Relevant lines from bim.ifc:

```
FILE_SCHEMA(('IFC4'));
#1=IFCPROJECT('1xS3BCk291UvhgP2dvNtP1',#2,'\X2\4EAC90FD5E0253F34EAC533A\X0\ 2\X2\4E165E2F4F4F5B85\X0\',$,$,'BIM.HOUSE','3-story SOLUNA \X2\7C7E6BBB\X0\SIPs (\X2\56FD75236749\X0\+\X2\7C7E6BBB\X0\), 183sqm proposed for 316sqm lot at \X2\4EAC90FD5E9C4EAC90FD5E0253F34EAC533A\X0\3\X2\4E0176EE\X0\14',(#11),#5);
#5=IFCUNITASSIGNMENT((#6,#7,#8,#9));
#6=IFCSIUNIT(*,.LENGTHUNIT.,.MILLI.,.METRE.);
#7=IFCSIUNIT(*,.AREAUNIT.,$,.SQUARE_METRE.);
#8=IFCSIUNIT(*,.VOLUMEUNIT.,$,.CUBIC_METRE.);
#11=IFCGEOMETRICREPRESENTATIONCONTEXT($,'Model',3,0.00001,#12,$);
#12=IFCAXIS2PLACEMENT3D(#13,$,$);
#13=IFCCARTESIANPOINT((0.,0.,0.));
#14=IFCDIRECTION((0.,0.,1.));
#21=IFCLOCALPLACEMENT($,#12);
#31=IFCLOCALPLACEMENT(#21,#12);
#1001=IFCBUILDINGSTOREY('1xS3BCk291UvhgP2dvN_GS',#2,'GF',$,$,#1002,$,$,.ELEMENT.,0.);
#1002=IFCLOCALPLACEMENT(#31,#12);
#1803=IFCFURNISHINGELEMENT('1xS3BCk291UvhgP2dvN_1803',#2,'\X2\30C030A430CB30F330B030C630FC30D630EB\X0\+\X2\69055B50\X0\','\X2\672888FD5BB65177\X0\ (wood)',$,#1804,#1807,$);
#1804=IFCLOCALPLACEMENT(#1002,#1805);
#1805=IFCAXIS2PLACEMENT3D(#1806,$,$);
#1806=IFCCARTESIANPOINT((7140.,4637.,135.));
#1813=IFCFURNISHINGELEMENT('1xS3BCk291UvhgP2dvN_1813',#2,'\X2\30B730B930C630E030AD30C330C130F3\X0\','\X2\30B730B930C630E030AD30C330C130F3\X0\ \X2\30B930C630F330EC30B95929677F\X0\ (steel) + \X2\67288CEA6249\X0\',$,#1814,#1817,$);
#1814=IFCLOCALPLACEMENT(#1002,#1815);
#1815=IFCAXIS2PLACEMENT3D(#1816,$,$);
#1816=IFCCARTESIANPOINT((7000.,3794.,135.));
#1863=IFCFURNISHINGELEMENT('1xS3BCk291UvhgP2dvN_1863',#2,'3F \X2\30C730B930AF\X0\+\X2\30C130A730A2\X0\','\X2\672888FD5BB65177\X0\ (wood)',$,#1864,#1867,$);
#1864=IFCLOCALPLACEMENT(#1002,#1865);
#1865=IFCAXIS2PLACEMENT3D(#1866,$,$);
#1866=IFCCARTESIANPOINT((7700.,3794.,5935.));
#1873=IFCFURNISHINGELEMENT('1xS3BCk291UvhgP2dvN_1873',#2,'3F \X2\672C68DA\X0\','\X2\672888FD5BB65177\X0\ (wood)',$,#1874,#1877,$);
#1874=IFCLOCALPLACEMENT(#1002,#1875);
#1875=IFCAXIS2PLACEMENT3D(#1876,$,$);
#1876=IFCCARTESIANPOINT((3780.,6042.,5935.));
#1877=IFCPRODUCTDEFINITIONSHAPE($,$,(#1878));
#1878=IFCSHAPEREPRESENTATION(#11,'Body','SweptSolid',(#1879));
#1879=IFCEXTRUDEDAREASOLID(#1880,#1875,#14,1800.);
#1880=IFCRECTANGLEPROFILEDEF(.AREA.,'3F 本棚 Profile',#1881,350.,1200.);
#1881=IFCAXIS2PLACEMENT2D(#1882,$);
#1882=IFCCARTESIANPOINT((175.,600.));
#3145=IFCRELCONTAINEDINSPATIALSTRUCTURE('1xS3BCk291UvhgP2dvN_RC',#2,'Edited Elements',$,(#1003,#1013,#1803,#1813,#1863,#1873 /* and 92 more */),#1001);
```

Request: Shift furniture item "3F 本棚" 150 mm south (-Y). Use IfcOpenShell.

```python
import ifcopenshell
import ifcopenshell.api.geometry
import ifcopenshell.util.placement

model = ifcopenshell.open("bim.ifc")

item = model.by_guid("1xS3BCk291UvhgP2dvN_1873")
matrix = ifcopenshell.util.placement.get_local_placement(item.ObjectPlacement)
matrix[1, 3] -= 150.0
ifcopenshell.api.geometry.edit_object_placement(model, product=item, matrix=matrix, is_si=False)

print(ifcopenshell.util.placement.get_local_placement(item.ObjectPlacement).round(3) + 0.0)

model.write("bim_updated.ifc")
```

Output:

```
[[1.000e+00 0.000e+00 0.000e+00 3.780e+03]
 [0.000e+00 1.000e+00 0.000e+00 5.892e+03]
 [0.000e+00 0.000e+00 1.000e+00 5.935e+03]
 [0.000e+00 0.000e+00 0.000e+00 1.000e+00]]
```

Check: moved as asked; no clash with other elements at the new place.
